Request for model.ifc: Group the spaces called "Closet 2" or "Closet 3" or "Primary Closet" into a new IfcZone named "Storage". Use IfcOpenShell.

First a look at what the model holds.

```python
import ifcopenshell

model = ifcopenshell.open("model.ifc")
print(model.schema)
seen = {}
for space in model.by_type("IfcSpace"):
    seen[space.LongName] = seen.get(space.LongName, 0) + 1
for name, count in sorted(seen.items(), key=str):
    print(count, "x", name)
print("zones:", [z.Name for z in model.by_type("IfcZone")][:20])
```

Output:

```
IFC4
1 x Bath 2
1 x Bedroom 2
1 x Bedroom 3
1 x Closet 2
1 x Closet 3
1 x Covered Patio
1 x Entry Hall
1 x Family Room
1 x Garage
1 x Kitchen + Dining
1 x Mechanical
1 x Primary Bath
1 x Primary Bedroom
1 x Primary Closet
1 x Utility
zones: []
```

```python
import ifcopenshell
import ifcopenshell.api.group
import ifcopenshell.api.root

model = ifcopenshell.open("model.ifc")

names = {"Closet 2", "Closet 3", "Primary Closet"}
spaces = [s for s in model.by_type("IfcSpace") if s.LongName in names]

zone = ifcopenshell.api.root.create_entity(model, ifc_class="IfcZone", name="Storage")
ifcopenshell.api.group.assign_group(model, products=spaces, group=zone)
print(len(spaces), "spaces in", zone.Name)

model.write("model_v2.ifc")
```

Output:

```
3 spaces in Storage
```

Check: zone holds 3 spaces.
